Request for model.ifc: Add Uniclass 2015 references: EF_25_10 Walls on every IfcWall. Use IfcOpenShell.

First a look at what the model holds.

```python
import ifcopenshell

model = ifcopenshell.open("model.ifc")
print(model.schema)
print("classifications:", [c.Name for c in model.by_type("IfcClassification")])
for ifc_class in ("IfcDoor", "IfcRoof", "IfcStair", "IfcWall", "IfcWindow"):
    print(ifc_class, len(model.by_type(ifc_class)))
```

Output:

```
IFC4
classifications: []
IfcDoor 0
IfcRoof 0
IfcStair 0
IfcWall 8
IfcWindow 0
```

```python
import ifcopenshell
import ifcopenshell.api.classification

model = ifcopenshell.open("model.ifc")

system = ifcopenshell.api.classification.add_classification(model, classification="Uniclass 2015")

codes = {
    "IfcWall": ("EF_25_10", "Walls"),
}
for ifc_class, (code, name) in codes.items():
    products = model.by_type(ifc_class)
    ifcopenshell.api.classification.add_reference(
        model, products=products, classification=system, identification=code, name=name
    )
    print(code, len(products))

model.write("model_rev.ifc")
```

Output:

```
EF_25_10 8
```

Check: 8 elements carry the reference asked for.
